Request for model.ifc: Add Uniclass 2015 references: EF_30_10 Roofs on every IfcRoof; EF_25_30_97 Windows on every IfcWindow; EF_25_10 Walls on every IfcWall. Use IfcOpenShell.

First a look at what the model holds.

```python
import ifcopenshell

model = ifcopenshell.open("model.ifc")
print(model.schema)
print("classifications:", [c.Name for c in model.by_type("IfcClassification")])
for ifc_class in ("IfcDoor", "IfcRoof", "IfcStair", "IfcWall", "IfcWindow"):
    print(ifc_class, len(model.by_type(ifc_class)))
```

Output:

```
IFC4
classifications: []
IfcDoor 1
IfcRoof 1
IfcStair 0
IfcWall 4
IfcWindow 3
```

```python
import ifcopenshell
import ifcopenshell.api.classification

model = ifcopenshell.open("model.ifc")

system = ifcopenshell.api.classification.add_classification(model, classification="Uniclass 2015")

codes = {
    "IfcRoof": ("EF_30_10", "Roofs"),
    "IfcWindow": ("EF_25_30_97", "Windows"),
    "IfcWall": ("EF_25_10", "Walls"),
}
for ifc_class, (code, name) in codes.items():
    products = model.by_type(ifc_class)
    ifcopenshell.api.classification.add_reference(
        model, products=products, classification=system, identification=code, name=name
    )
    print(code, len(products))

model.write("model_v2.ifc")
```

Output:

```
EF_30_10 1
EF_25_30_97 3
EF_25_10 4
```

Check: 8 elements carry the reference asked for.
